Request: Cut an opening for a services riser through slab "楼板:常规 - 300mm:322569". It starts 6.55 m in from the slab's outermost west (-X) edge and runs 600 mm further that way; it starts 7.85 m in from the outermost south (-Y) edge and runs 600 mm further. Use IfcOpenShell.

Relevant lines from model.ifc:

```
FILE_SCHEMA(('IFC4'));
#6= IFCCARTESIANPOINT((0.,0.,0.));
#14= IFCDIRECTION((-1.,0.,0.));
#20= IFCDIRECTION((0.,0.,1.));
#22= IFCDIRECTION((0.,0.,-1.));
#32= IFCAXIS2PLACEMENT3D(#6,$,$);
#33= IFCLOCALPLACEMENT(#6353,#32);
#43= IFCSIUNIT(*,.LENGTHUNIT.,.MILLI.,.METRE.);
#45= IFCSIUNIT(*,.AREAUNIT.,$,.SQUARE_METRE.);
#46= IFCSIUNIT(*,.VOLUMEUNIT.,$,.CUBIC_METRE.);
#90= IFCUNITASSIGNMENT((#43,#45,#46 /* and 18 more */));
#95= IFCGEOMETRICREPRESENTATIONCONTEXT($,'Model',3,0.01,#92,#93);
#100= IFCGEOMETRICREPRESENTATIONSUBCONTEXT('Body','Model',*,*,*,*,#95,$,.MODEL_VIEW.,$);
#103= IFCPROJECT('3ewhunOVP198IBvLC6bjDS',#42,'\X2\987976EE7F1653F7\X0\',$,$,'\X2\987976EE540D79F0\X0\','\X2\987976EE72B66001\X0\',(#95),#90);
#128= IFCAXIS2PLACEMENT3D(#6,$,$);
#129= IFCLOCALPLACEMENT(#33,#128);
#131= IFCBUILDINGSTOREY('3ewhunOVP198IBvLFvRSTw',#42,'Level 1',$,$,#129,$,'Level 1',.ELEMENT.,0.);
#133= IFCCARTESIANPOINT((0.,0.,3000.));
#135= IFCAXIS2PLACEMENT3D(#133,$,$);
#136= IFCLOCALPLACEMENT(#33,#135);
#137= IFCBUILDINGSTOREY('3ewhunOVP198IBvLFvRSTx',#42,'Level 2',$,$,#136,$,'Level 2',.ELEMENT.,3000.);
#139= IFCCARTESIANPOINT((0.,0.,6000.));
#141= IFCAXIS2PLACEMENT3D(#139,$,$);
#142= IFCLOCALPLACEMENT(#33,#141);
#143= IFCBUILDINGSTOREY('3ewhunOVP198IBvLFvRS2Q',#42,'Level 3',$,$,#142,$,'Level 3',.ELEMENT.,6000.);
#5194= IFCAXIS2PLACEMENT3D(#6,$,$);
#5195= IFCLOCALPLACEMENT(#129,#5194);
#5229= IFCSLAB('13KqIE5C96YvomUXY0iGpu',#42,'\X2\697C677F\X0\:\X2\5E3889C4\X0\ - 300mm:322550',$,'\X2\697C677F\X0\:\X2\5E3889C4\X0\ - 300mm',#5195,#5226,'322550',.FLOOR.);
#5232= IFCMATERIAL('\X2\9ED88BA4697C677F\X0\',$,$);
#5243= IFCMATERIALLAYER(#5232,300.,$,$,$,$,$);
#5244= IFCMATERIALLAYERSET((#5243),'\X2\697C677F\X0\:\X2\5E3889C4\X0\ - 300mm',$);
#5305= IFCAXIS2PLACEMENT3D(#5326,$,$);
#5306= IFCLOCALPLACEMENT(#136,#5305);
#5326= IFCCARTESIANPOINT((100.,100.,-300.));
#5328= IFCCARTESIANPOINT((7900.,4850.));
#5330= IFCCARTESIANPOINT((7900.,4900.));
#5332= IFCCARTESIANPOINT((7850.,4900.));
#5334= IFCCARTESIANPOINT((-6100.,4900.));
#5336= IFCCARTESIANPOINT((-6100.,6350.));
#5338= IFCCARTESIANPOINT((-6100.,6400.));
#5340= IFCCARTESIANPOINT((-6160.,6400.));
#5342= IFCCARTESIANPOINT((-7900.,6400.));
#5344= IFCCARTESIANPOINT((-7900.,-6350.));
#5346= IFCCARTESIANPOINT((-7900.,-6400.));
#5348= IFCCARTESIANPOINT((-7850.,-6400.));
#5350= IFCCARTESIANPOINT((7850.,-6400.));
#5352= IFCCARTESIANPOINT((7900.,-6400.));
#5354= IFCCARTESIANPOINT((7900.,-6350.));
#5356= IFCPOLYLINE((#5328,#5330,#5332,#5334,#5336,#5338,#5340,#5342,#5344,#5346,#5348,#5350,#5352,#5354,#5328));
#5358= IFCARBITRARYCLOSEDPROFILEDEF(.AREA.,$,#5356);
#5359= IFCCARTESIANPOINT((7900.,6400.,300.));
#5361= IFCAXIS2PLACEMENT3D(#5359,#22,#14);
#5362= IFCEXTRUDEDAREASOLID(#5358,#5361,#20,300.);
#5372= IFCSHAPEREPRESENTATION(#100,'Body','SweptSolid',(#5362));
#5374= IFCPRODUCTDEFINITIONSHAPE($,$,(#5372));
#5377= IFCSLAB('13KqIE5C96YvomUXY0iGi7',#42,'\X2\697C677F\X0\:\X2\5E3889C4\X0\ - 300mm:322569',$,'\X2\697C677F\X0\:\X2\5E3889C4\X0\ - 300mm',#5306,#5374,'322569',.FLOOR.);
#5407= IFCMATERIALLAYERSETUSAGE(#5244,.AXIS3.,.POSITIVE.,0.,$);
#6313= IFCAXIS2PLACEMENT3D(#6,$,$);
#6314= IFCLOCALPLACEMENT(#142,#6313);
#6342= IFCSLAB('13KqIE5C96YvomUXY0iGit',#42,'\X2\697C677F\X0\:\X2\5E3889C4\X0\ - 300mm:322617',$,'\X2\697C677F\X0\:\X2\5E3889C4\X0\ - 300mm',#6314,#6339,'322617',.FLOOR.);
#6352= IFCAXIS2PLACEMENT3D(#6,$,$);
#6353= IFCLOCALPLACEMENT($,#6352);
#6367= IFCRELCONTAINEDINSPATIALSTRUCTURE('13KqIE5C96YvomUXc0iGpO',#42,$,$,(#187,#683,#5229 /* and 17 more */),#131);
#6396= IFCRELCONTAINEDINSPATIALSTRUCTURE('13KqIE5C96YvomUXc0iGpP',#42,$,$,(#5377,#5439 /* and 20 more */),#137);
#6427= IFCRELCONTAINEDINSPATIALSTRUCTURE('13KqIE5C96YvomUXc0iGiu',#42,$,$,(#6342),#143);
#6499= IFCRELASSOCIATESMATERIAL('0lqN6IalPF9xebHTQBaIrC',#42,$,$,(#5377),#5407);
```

```python
import numpy as np
import ifcopenshell
import ifcopenshell.api.feature
import ifcopenshell.api.geometry
import ifcopenshell.api.root
import ifcopenshell.geom
import ifcopenshell.util.placement
import ifcopenshell.util.representation
import ifcopenshell.util.shape
import ifcopenshell.util.unit

model = ifcopenshell.open("model.ifc")
unit_scale = ifcopenshell.util.unit.calculate_unit_scale(model)
settings = ifcopenshell.geom.settings()


def volume(element):
    """Net volume in cubic metres, openings subtracted."""
    shape = ifcopenshell.geom.create_shape(settings, element)
    return ifcopenshell.util.shape.get_volume(shape.geometry)


slab = model.by_guid("13KqIE5C96YvomUXY0iGi7")
before = volume(slab)

# Extent in the slab's own axes, in metres. The edges named are its -X and -Y sides.
slab_shape = ifcopenshell.geom.create_shape(settings, slab)
vertices = ifcopenshell.util.shape.get_vertices(slab_shape.geometry)
x_min, y_min, bottom = vertices.min(axis=0)
top = vertices[:, 2].max()

opening = ifcopenshell.api.root.create_entity(model, ifc_class="IfcOpeningElement", name="Services riser opening", predefined_type="OPENING")
context = ifcopenshell.util.representation.get_context(model, "Model", "Body", "MODEL_VIEW")
width, depth = 0.6, 0.6
outline = [(0.0, 0.0), (width, 0.0), (width, depth), (0.0, depth), (0.0, 0.0)]
# Overshoot both faces by 50 mm so the cut is clean.
shape = ifcopenshell.api.geometry.add_slab_representation(
    model, context=context, depth=top - bottom + 0.1, polyline=outline
)
ifcopenshell.api.geometry.assign_representation(model, product=opening, representation=shape)

matrix = ifcopenshell.util.placement.get_local_placement(slab.ObjectPlacement)
matrix[:, 3] = matrix @ np.append(np.array([x_min + 6.55, y_min + 7.85, bottom - 0.05]) / unit_scale, 1.0)
ifcopenshell.api.geometry.edit_object_placement(model, product=opening, matrix=matrix, is_si=False)
ifcopenshell.api.feature.add_feature(model, feature=opening, element=slab)

after = volume(slab)

print(f"slab volume {before:.3f} -> {after:.3f} m3")

model.write("model_rev.ifc")
```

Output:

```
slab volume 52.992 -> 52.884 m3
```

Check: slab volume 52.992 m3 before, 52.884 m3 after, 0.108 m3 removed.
